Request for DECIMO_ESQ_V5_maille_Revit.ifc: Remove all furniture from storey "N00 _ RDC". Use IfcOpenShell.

First a look at what the model holds.

```python
import ifcopenshell
import ifcopenshell.util.element

model = ifcopenshell.open("DECIMO_ESQ_V5_maille_Revit.ifc")
print(model.schema)
storey = next(s for s in model.by_type("IfcBuildingStorey") if s.Name == "N00 _ RDC")
furniture = [e for e in ifcopenshell.util.element.get_decomposition(storey) if e.is_a("IfcFurnishingElement")]
seen = {}
for e in furniture:
    element_type = ifcopenshell.util.element.get_type(e)
    name = element_type.Name if element_type not in (None, e) else None
    seen[name] = seen.get(name, 0) + 1
for name, count in sorted(seen.items(), key=str):
    print(count, "x", name)
```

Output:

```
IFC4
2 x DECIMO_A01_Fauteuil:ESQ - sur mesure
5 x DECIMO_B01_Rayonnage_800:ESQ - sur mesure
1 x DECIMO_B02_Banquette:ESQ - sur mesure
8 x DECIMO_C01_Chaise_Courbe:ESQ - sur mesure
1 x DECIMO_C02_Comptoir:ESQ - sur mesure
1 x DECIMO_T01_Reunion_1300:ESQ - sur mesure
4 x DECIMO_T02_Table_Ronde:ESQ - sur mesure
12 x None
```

```python
import ifcopenshell
import ifcopenshell.api.root
import ifcopenshell.util.element

model = ifcopenshell.open("DECIMO_ESQ_V5_maille_Revit.ifc")

storey = next(s for s in model.by_type("IfcBuildingStorey") if s.Name == "N00 _ RDC")
furniture = [e for e in ifcopenshell.util.element.get_decomposition(storey) if e.is_a("IfcFurnishingElement")]

for e in furniture:
    ifcopenshell.api.root.remove_product(model, product=e)
print(len(furniture), "removed")

model.write("DECIMO_ESQ_V5_maille_Revit_updated.ifc")
```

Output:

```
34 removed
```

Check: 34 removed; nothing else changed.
